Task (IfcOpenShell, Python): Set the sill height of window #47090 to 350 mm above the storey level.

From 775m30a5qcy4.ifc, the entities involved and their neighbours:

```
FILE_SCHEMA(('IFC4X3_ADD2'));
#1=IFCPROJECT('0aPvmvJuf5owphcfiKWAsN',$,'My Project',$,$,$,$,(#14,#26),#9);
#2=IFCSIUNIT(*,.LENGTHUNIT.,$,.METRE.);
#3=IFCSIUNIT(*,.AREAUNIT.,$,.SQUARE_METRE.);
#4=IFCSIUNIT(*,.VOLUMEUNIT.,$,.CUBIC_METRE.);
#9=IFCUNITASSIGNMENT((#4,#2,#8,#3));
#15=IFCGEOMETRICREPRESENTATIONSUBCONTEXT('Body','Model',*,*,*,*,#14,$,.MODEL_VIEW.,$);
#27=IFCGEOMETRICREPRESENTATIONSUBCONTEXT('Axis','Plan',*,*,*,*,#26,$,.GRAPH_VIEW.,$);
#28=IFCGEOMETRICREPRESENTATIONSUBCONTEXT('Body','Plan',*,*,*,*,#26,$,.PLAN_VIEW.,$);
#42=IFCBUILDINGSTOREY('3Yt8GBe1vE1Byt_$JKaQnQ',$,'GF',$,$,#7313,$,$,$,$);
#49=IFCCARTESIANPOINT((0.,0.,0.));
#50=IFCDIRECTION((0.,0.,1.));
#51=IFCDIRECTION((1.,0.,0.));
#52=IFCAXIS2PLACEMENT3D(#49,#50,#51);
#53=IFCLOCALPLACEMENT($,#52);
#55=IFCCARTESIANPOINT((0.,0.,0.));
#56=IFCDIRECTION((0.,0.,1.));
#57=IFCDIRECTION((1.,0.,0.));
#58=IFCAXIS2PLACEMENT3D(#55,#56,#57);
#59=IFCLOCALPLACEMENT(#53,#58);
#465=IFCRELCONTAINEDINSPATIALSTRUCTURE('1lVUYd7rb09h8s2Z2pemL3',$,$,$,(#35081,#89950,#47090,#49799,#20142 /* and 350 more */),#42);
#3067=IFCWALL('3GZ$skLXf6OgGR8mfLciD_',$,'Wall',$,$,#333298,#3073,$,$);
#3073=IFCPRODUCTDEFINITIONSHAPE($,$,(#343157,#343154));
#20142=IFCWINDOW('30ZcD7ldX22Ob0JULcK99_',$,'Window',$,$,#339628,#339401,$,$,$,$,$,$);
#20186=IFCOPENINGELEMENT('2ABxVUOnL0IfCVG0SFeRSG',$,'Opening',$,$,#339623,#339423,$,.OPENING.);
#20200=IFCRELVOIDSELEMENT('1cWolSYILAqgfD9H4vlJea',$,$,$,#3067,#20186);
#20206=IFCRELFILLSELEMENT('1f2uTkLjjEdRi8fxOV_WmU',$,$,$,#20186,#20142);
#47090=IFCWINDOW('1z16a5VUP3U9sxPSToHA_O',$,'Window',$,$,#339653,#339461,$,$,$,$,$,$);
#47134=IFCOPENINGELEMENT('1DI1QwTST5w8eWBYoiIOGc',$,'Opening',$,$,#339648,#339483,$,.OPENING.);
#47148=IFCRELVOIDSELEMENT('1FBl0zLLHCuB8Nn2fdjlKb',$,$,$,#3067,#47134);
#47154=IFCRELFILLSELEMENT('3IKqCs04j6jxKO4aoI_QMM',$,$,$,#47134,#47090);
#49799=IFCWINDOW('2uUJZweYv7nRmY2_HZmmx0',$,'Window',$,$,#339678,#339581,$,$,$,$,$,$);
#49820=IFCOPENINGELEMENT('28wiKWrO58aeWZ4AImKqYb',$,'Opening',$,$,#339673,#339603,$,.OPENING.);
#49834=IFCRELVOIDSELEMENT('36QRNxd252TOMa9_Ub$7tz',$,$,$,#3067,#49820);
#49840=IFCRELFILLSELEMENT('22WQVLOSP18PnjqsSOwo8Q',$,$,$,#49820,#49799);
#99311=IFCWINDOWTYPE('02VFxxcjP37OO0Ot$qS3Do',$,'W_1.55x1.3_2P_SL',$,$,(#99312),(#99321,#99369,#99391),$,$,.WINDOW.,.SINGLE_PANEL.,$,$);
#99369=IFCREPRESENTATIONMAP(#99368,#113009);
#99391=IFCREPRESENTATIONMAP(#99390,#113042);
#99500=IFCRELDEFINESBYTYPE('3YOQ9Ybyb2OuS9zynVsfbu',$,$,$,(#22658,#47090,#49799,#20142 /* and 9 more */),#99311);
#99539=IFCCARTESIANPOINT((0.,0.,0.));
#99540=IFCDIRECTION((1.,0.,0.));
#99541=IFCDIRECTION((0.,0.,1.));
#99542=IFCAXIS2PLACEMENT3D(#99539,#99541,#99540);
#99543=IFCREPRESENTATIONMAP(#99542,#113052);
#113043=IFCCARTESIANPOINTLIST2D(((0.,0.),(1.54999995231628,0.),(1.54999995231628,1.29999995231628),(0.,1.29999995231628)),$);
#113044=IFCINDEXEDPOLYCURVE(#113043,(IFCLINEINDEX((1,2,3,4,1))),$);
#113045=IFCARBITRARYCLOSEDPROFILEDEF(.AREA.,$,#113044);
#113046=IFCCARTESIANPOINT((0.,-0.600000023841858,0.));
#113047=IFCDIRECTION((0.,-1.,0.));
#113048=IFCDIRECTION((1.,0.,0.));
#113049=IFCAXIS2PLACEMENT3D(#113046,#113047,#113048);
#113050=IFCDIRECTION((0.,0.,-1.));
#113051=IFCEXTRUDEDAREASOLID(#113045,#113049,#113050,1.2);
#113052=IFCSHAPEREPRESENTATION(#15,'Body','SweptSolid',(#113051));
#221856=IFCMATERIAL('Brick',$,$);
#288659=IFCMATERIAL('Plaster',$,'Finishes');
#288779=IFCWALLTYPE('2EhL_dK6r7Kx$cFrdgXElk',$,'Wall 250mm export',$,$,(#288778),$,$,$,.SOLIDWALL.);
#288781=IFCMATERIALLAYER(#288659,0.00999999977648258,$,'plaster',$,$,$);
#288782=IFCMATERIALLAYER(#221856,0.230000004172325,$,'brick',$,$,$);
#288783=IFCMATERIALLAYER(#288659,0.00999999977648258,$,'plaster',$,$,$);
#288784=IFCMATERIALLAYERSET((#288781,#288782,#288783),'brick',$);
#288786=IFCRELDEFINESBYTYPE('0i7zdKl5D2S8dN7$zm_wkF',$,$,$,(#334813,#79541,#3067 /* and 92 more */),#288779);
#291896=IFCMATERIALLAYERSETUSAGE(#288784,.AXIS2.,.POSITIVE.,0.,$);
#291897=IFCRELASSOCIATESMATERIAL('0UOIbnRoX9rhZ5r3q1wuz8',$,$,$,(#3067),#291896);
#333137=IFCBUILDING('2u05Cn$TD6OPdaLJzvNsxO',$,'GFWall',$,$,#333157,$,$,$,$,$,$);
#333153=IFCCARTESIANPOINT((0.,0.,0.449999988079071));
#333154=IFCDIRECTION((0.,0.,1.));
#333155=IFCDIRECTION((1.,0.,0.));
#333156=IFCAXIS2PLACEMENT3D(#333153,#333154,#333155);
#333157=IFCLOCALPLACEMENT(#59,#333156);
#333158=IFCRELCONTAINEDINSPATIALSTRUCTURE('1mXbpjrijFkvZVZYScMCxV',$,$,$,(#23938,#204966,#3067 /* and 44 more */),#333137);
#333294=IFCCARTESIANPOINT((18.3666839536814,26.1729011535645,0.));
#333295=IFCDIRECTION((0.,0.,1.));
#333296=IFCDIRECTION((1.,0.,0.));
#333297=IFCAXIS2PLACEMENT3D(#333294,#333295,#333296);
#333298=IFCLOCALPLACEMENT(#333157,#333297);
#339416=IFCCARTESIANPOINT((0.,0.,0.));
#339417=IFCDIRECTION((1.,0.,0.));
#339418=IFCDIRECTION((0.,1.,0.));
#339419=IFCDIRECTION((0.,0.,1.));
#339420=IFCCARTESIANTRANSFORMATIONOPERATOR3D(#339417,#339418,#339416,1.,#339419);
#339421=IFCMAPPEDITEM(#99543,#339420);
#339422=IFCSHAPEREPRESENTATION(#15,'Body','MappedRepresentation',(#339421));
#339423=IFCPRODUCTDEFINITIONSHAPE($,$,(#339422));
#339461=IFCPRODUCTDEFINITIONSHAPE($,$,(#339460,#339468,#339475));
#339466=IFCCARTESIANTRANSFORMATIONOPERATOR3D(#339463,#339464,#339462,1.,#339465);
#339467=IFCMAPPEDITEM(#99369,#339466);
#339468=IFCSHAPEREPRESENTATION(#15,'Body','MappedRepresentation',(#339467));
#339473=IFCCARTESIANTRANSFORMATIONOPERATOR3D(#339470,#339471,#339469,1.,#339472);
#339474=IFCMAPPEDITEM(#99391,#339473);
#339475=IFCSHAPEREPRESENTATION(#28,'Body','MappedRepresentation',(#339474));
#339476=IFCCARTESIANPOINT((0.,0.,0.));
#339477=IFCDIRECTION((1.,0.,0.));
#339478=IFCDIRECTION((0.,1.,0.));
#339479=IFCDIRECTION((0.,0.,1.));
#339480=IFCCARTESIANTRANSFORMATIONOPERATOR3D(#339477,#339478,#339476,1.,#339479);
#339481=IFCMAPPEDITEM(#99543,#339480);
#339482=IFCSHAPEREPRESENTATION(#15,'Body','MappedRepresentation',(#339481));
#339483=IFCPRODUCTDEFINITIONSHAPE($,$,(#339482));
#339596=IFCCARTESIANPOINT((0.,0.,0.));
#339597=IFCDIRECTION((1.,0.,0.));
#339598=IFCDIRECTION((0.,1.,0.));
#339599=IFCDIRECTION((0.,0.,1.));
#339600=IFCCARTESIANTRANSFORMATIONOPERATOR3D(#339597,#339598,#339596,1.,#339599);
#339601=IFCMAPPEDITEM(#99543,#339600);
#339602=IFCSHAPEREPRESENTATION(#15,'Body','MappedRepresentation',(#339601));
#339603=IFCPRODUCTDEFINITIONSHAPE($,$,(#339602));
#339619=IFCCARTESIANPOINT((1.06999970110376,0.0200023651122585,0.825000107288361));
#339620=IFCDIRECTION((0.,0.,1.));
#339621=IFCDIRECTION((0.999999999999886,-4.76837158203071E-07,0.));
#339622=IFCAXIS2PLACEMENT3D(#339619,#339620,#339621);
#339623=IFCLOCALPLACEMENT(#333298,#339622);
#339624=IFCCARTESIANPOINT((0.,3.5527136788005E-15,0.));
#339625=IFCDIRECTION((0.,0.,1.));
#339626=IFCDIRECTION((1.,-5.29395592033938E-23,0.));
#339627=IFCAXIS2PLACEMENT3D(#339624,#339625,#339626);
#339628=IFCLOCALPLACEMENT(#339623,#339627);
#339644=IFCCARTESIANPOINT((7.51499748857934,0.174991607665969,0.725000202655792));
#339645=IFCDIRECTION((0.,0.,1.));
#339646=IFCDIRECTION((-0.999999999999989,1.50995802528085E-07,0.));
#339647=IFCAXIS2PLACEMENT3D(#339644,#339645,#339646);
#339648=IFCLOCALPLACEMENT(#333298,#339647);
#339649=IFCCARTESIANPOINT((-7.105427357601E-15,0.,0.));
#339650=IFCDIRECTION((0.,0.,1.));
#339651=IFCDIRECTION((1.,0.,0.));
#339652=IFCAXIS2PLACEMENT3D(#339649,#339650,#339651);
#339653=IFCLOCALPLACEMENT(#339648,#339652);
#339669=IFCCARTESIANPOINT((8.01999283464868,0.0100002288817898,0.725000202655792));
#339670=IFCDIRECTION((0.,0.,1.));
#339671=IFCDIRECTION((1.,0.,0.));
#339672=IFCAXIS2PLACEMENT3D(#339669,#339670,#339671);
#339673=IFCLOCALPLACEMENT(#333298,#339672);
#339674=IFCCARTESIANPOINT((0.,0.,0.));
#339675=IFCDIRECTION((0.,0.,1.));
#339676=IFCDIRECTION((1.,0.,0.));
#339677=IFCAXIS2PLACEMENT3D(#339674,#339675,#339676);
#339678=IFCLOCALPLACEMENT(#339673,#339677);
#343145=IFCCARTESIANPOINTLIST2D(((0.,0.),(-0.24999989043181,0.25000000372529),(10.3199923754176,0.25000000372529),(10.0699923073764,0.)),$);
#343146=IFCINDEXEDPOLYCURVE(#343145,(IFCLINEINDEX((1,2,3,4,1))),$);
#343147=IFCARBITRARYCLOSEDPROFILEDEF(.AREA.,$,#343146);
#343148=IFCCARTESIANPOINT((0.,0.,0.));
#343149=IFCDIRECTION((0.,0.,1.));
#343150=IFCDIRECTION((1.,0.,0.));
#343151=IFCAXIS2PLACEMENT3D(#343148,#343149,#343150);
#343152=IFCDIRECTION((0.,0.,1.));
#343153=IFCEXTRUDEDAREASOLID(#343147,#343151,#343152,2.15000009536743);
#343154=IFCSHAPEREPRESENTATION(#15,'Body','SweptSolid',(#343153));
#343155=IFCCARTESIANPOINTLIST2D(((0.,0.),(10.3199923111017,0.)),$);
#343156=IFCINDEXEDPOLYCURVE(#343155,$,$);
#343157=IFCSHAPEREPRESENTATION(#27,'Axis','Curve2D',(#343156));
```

```python
import numpy as np
import ifcopenshell
import ifcopenshell.api.geometry
import ifcopenshell.geom
import ifcopenshell.util.element
import ifcopenshell.util.placement
import ifcopenshell.util.shape
import ifcopenshell.util.unit

model = ifcopenshell.open("775m30a5qcy4.ifc")
unit_scale = ifcopenshell.util.unit.calculate_unit_scale(model)

window = model.by_guid("1z16a5VUP3U9sxPSToHA_O")
opening = window.FillsVoids[0].RelatingOpeningElement
storey = ifcopenshell.util.element.get_container(window, ifc_class="IfcBuildingStorey")
level = ifcopenshell.util.placement.get_local_placement(storey.ObjectPlacement)[2, 3]

# The opening's origin need not be at the sill, so measure its lowest point.
shape = ifcopenshell.geom.create_shape(ifcopenshell.geom.settings(), opening)
bottom = ifcopenshell.util.shape.get_shape_bottom_elevation(shape, shape.geometry) / unit_scale
dz = level + 0.35 / unit_scale - bottom

shift = np.array([0.0, 0.0, dz])
# The window is placed relative to its opening, so it follows when the opening moves.
matrix = ifcopenshell.util.placement.get_local_placement(opening.ObjectPlacement)
matrix[:3, 3] += shift
ifcopenshell.api.geometry.edit_object_placement(
    model, product=opening, matrix=matrix, is_si=False, should_transform_children=True
)

print(f"moved by {dz * unit_scale:+.3f} m")

model.write("775m30a5qcy4_v2.ifc")
```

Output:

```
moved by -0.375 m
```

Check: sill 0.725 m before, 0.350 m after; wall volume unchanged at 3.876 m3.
